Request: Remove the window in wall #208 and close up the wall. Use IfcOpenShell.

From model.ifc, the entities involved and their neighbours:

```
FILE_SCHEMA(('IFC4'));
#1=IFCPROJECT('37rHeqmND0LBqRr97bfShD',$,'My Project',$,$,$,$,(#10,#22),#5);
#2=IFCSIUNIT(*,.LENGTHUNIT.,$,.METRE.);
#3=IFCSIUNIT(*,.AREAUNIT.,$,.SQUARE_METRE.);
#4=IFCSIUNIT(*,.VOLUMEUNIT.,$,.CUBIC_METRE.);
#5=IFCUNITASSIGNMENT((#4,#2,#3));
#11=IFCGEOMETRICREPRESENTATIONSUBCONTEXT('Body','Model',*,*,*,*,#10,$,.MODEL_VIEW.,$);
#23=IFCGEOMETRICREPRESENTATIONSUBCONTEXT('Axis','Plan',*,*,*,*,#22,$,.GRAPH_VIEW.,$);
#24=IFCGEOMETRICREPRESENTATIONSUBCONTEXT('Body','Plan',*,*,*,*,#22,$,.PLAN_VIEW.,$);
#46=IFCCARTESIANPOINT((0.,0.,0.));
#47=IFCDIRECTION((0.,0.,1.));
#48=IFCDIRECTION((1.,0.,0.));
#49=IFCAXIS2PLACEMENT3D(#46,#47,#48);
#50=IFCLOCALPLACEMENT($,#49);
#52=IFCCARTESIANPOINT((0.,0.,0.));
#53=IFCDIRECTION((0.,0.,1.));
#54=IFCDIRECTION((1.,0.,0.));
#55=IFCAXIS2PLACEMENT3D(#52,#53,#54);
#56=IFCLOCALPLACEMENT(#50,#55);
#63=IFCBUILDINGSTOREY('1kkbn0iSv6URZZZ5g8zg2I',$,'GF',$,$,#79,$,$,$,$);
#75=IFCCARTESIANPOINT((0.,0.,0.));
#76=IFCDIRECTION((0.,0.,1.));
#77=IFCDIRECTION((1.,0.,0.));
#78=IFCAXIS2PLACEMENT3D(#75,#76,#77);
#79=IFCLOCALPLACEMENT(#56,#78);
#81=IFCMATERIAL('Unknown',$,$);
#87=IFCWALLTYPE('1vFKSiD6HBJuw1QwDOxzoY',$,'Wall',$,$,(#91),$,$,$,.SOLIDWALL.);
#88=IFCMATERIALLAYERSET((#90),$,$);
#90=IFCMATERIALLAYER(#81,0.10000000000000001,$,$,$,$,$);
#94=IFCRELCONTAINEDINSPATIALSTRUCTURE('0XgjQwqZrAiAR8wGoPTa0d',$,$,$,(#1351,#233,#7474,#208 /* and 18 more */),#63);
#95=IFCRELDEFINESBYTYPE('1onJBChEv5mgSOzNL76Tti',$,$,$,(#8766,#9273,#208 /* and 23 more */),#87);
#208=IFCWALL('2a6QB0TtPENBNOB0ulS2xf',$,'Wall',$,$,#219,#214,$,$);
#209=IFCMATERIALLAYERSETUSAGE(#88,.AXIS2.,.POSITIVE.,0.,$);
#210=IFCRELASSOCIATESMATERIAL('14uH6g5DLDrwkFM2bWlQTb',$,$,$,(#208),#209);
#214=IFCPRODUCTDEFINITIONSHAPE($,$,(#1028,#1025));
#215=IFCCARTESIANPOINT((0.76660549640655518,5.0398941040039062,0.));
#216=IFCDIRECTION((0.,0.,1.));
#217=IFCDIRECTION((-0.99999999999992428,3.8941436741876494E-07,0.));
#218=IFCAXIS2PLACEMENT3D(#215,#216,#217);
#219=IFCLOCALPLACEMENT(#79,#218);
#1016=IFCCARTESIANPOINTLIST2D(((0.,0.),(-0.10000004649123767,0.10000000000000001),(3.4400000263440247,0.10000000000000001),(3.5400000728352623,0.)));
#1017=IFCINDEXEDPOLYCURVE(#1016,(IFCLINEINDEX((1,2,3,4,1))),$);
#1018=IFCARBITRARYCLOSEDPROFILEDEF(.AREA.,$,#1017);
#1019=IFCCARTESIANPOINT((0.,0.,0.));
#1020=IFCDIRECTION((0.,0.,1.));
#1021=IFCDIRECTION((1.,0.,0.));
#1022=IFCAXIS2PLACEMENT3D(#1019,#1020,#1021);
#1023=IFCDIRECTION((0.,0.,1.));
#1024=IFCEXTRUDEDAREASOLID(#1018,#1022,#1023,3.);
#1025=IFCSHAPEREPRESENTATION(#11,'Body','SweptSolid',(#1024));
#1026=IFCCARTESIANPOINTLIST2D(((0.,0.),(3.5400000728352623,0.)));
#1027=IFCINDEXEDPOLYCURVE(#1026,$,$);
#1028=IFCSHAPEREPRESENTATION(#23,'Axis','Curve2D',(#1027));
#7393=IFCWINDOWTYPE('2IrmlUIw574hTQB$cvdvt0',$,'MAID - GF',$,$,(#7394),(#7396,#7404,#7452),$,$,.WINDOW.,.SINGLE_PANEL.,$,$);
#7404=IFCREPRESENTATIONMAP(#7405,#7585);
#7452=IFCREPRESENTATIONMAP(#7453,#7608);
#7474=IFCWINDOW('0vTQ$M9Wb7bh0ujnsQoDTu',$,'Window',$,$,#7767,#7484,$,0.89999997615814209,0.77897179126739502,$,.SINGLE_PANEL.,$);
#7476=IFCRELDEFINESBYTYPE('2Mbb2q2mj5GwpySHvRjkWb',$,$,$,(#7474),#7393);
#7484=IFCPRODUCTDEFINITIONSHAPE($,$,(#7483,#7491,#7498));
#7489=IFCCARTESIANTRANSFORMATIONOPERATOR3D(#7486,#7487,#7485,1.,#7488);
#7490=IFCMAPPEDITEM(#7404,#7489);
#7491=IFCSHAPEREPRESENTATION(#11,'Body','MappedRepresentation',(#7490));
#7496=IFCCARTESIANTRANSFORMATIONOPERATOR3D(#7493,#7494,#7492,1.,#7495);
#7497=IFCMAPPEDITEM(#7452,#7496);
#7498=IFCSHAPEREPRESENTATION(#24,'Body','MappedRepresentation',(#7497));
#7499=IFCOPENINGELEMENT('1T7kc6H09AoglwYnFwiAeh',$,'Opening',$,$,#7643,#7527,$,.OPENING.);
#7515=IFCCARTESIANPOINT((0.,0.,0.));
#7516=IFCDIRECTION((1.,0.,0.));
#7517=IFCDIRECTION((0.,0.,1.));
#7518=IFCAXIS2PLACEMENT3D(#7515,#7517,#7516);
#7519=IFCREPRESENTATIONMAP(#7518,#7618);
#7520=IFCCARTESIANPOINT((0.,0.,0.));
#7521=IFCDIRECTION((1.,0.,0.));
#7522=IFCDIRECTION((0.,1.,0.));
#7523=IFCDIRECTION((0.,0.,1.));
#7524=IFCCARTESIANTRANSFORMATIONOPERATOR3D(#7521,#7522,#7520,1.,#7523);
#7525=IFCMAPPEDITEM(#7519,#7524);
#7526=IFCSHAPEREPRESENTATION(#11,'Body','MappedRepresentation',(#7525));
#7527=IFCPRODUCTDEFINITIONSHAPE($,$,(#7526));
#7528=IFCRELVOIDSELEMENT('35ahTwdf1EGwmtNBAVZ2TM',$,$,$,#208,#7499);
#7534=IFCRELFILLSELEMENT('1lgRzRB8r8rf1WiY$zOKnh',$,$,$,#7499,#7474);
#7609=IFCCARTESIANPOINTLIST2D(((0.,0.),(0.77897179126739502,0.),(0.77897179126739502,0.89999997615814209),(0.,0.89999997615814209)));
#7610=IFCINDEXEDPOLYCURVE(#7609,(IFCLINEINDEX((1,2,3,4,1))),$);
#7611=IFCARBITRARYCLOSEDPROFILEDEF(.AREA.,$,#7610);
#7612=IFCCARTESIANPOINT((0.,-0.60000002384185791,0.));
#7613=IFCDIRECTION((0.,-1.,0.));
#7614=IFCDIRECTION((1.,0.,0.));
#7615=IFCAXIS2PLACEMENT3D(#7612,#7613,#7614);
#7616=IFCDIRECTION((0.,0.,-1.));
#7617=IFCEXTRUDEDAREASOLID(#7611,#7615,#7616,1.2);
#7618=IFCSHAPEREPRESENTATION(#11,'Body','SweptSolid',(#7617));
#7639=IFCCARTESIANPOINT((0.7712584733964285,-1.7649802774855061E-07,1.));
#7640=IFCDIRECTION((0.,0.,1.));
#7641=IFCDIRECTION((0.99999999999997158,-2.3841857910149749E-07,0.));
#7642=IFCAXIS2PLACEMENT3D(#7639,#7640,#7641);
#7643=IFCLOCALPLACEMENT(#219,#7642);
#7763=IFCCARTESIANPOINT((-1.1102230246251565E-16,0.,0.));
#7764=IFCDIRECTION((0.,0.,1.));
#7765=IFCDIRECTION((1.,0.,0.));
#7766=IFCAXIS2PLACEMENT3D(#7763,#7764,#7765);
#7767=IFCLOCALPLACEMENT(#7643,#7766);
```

```python
import ifcopenshell
import ifcopenshell.api.feature
import ifcopenshell.api.root
import ifcopenshell.geom
import ifcopenshell.util.shape

model = ifcopenshell.open("model.ifc")
settings = ifcopenshell.geom.settings()


def volume(element):
    """Net volume in cubic metres, openings subtracted."""
    shape = ifcopenshell.geom.create_shape(settings, element)
    return ifcopenshell.util.shape.get_volume(shape.geometry)


window = model.by_id(7474)
opening = window.FillsVoids[0].RelatingOpeningElement
wall = opening.VoidsElements[0].RelatingBuildingElement
before = volume(wall)

ifcopenshell.api.root.remove_product(model, product=window)
ifcopenshell.api.feature.remove_feature(model, feature=opening)

after = volume(wall)

print(f"wall volume {before:.3f} -> {after:.3f} m3")

model.write("model_rev.ifc")
```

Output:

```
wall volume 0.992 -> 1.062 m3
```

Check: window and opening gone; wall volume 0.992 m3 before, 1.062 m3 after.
